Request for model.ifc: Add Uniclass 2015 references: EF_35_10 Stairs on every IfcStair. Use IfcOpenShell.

First a look at what the model holds.

```python
import ifcopenshell

model = ifcopenshell.open("model.ifc")
print(model.schema)
print("classifications:", [c.Name for c in model.by_type("IfcClassification")])
for ifc_class in ("IfcDoor", "IfcRoof", "IfcStair", "IfcWall", "IfcWindow"):
    print(ifc_class, len(model.by_type(ifc_class)))
```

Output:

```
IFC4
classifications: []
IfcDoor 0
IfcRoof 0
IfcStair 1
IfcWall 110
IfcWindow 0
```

```python
import ifcopenshell
import ifcopenshell.api.classification

model = ifcopenshell.open("model.ifc")

system = ifcopenshell.api.classification.add_classification(model, classification="Uniclass 2015")

codes = {
    "IfcStair": ("EF_35_10", "Stairs"),
}
for ifc_class, (code, name) in codes.items():
    products = model.by_type(ifc_class)
    ifcopenshell.api.classification.add_reference(
        model, products=products, classification=system, identification=code, name=name
    )
    print(code, len(products))

model.write("model_edited.ifc")
```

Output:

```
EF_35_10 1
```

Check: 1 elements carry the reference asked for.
